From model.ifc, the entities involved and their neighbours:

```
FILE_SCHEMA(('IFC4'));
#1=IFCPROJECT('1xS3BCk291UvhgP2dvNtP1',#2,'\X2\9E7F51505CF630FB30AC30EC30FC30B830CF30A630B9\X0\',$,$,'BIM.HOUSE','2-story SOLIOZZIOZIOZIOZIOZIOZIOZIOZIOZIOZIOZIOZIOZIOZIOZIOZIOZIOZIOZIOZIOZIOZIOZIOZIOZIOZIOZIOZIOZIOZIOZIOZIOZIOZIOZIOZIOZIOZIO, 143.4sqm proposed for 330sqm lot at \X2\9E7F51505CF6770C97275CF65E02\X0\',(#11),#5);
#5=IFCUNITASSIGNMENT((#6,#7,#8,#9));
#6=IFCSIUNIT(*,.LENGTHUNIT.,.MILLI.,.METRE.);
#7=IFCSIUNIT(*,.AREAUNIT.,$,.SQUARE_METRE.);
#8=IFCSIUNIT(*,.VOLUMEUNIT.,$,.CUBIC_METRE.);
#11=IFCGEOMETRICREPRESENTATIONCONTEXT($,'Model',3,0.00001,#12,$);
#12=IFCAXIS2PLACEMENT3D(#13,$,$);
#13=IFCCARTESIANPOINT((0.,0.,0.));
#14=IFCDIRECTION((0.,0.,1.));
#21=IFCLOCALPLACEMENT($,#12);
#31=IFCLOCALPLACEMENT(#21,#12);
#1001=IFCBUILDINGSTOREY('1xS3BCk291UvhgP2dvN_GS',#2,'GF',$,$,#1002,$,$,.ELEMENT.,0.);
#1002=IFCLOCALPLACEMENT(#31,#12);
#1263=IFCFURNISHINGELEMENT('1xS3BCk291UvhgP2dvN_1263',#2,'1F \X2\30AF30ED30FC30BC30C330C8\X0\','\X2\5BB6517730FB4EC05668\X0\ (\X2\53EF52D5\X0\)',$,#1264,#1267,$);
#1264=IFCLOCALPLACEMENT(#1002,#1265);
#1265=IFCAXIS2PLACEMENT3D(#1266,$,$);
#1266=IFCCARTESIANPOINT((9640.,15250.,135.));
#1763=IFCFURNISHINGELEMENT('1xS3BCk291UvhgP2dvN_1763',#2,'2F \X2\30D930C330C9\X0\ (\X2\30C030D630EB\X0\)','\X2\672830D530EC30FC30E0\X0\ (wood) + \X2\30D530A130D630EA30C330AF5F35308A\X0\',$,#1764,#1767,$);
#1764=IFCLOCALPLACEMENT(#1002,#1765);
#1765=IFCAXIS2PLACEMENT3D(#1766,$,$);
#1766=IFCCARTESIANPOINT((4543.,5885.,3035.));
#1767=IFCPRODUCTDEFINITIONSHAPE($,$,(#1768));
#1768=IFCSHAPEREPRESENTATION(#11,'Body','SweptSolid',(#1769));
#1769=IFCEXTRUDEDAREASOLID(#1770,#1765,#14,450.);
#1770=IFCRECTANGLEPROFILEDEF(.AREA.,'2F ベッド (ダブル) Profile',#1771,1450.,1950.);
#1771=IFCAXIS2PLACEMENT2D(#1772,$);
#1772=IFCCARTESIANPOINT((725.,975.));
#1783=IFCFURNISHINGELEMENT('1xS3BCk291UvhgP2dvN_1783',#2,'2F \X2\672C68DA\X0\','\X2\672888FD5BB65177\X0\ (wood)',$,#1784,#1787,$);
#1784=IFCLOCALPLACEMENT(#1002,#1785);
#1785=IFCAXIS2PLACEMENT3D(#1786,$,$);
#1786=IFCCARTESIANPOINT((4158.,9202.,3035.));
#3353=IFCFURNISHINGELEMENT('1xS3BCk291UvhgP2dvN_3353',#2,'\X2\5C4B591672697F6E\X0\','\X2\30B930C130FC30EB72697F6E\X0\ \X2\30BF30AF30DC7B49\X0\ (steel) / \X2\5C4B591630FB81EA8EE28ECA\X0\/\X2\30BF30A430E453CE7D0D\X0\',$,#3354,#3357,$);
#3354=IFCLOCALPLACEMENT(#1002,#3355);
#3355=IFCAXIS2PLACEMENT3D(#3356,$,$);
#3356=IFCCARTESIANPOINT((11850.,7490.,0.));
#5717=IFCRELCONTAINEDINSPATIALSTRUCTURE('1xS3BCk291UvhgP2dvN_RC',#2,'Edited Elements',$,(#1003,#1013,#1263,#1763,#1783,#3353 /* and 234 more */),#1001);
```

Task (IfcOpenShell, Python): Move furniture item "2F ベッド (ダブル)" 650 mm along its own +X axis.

```python
import ifcopenshell
import ifcopenshell.api.geometry
import ifcopenshell.util.placement
import ifcopenshell.util.unit

model = ifcopenshell.open("model.ifc")
unit_scale = ifcopenshell.util.unit.calculate_unit_scale(model)

item = model.by_id(1763)
matrix = ifcopenshell.util.placement.get_local_placement(item.ObjectPlacement)
matrix[:3, 3] += matrix[:3, 0] * 0.65 / unit_scale
ifcopenshell.api.geometry.edit_object_placement(model, product=item, matrix=matrix, is_si=False)

print(ifcopenshell.util.placement.get_local_placement(item.ObjectPlacement).round(3) + 0.0)

model.write("model_v2.ifc")
```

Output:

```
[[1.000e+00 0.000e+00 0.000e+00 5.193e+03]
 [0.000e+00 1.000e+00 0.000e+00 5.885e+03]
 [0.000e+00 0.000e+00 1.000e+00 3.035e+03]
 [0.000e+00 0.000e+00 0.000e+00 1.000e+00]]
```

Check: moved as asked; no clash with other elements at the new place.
